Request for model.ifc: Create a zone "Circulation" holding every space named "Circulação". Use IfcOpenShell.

First a look at what the model holds.

```python
import ifcopenshell

model = ifcopenshell.open("model.ifc")
print(model.schema)
seen = {}
for space in model.by_type("IfcSpace"):
    seen[space.LongName] = seen.get(space.LongName, 0) + 1
for name, count in sorted(seen.items(), key=str):
    print(count, "x", name)
print("zones:", [z.Name for z in model.by_type("IfcZone")][:20])
```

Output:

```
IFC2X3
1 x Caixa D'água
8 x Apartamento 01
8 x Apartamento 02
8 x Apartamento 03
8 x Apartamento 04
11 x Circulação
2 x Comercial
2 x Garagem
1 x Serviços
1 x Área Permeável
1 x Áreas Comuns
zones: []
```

```python
import ifcopenshell
import ifcopenshell.api.group
import ifcopenshell.api.root

model = ifcopenshell.open("model.ifc")

names = {"Circulação"}
spaces = [s for s in model.by_type("IfcSpace") if s.LongName in names]

zone = ifcopenshell.api.root.create_entity(model, ifc_class="IfcZone", name="Circulation")
ifcopenshell.api.group.assign_group(model, products=spaces, group=zone)
print(len(spaces), "spaces in", zone.Name)

model.write("model-out.ifc")
```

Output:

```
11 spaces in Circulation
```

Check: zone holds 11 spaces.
